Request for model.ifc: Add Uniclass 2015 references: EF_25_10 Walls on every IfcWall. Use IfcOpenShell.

First a look at what the model holds.

```python
import ifcopenshell

model = ifcopenshell.open("model.ifc")
print(model.schema)
print("classifications:", [c.Name for c in model.by_type("IfcClassification")])
for ifc_class in ("IfcDoor", "IfcRoof", "IfcStair", "IfcWall", "IfcWindow"):
    print(ifc_class, len(model.by_type(ifc_class)))
```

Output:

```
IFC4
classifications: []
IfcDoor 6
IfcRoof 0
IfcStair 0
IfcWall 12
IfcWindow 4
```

```python
import ifcopenshell
import ifcopenshell.api.classification

model = ifcopenshell.open("model.ifc")

system = ifcopenshell.api.classification.add_classification(model, classification="Uniclass 2015")

codes = {
    "IfcWall": ("EF_25_10", "Walls"),
}
for ifc_class, (code, name) in codes.items():
    products = model.by_type(ifc_class)
    ifcopenshell.api.classification.add_reference(
        model, products=products, classification=system, identification=code, name=name
    )
    print(code, len(products))

model.write("model_rev.ifc")
```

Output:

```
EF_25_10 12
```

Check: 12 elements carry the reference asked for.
